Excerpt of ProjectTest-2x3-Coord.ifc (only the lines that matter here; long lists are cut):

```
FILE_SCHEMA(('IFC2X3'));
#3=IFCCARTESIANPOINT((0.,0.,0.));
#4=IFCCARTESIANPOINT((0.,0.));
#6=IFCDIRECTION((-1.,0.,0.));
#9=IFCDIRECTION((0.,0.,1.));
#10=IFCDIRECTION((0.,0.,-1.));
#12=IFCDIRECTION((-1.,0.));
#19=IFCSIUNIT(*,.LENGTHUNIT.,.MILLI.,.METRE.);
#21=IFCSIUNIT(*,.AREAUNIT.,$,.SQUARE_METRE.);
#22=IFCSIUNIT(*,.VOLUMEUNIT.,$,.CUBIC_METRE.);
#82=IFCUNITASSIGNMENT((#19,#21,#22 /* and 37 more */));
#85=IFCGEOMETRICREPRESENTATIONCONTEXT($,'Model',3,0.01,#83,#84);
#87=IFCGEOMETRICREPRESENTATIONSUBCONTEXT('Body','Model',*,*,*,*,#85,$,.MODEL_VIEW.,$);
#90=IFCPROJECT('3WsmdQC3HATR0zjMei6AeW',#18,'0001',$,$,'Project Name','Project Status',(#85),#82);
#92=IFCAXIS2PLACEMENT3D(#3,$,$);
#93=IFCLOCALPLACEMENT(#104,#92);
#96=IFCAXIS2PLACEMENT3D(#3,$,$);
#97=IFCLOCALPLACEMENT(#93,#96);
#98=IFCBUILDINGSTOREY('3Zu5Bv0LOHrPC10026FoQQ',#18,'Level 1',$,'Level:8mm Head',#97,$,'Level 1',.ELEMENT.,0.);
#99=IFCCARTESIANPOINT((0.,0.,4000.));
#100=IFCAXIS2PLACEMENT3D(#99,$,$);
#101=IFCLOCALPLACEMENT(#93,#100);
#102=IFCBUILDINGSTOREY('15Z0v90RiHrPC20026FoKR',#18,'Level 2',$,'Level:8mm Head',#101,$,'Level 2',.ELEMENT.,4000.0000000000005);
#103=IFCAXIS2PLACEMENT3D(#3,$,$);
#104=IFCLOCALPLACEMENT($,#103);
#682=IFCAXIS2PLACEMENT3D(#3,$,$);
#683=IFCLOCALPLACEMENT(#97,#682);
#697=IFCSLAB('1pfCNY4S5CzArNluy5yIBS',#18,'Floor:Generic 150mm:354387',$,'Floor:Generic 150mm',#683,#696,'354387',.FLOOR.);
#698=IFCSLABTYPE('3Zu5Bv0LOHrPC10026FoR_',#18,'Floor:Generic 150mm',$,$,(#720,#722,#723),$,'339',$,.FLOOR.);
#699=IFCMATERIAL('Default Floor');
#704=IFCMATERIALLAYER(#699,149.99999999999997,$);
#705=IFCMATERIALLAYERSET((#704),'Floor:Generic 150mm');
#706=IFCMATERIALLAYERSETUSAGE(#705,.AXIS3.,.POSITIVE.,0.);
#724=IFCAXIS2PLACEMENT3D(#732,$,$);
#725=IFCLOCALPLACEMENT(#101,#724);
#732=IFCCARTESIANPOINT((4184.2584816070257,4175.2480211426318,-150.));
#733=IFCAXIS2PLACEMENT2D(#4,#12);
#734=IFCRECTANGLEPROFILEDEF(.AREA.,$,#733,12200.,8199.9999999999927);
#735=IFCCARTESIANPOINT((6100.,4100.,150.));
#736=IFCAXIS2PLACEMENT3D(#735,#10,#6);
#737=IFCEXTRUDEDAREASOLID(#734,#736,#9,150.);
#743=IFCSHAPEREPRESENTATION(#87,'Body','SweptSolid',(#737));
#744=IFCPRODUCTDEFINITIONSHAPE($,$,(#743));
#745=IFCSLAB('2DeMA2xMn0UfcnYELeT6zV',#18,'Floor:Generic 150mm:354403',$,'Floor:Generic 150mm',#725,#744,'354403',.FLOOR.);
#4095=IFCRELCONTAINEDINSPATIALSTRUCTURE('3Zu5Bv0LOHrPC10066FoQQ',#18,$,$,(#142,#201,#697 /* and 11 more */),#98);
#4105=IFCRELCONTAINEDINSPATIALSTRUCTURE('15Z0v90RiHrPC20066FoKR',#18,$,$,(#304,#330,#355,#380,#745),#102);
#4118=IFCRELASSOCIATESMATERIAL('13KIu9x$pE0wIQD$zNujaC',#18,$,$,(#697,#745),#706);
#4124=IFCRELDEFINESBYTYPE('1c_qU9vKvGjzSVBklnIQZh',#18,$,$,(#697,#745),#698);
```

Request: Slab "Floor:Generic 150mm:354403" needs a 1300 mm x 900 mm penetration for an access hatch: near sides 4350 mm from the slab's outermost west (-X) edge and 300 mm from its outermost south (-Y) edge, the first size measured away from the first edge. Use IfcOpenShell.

```python
import numpy as np
import ifcopenshell
import ifcopenshell.api.feature
import ifcopenshell.api.geometry
import ifcopenshell.api.root
import ifcopenshell.geom
import ifcopenshell.util.placement
import ifcopenshell.util.representation
import ifcopenshell.util.shape
import ifcopenshell.util.unit

model = ifcopenshell.open("ProjectTest-2x3-Coord.ifc")
unit_scale = ifcopenshell.util.unit.calculate_unit_scale(model)
settings = ifcopenshell.geom.settings()


def volume(element):
    """Net volume in cubic metres, openings subtracted."""
    shape = ifcopenshell.geom.create_shape(settings, element)
    return ifcopenshell.util.shape.get_volume(shape.geometry)


slab = model.by_guid("2DeMA2xMn0UfcnYELeT6zV")
before = volume(slab)

# Extent in the slab's own axes, in metres. The edges named are its -X and -Y sides.
slab_shape = ifcopenshell.geom.create_shape(settings, slab)
vertices = ifcopenshell.util.shape.get_vertices(slab_shape.geometry)
x_min, y_min, bottom = vertices.min(axis=0)
top = vertices[:, 2].max()

opening = ifcopenshell.api.root.create_entity(model, ifc_class="IfcOpeningElement", name="Access hatch opening")
context = ifcopenshell.util.representation.get_context(model, "Model", "Body", "MODEL_VIEW")
width, depth = 1.3, 0.9
outline = [(0.0, 0.0), (width, 0.0), (width, depth), (0.0, depth), (0.0, 0.0)]
# Overshoot both faces by 50 mm so the cut is clean.
shape = ifcopenshell.api.geometry.add_slab_representation(
    model, context=context, depth=top - bottom + 0.1, polyline=outline
)
ifcopenshell.api.geometry.assign_representation(model, product=opening, representation=shape)

matrix = ifcopenshell.util.placement.get_local_placement(slab.ObjectPlacement)
matrix[:, 3] = matrix @ np.append(np.array([x_min + 4.35, y_min + 0.3, bottom - 0.05]) / unit_scale, 1.0)
ifcopenshell.api.geometry.edit_object_placement(model, product=opening, matrix=matrix, is_si=False)
ifcopenshell.api.feature.add_feature(model, feature=opening, element=slab)

after = volume(slab)

print(f"slab volume {before:.3f} -> {after:.3f} m3")

model.write("ProjectTest-2x3-Coord_edited.ifc")
```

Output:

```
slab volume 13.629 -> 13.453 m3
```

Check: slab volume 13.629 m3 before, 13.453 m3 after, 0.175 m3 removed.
